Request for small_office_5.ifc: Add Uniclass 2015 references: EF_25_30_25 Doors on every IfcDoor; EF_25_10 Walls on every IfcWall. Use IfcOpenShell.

First a look at what the model holds.

```python
import ifcopenshell

model = ifcopenshell.open("small_office_5.ifc")
print(model.schema)
print("classifications:", [c.Name for c in model.by_type("IfcClassification")])
for ifc_class in ("IfcDoor", "IfcRoof", "IfcStair", "IfcWall", "IfcWindow"):
    print(ifc_class, len(model.by_type(ifc_class)))
```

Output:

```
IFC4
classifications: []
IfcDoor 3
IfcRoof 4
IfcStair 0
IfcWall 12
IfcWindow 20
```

```python
import ifcopenshell
import ifcopenshell.api.classification

model = ifcopenshell.open("small_office_5.ifc")

system = ifcopenshell.api.classification.add_classification(model, classification="Uniclass 2015")

codes = {
    "IfcDoor": ("EF_25_30_25", "Doors"),
    "IfcWall": ("EF_25_10", "Walls"),
}
for ifc_class, (code, name) in codes.items():
    products = model.by_type(ifc_class)
    ifcopenshell.api.classification.add_reference(
        model, products=products, classification=system, identification=code, name=name
    )
    print(code, len(products))

model.write("small_office_5_edited.ifc")
```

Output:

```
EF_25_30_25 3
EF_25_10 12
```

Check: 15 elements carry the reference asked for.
